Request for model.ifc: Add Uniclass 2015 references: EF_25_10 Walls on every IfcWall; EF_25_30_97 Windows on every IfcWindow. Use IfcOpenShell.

First a look at what the model holds.

```python
import ifcopenshell

model = ifcopenshell.open("model.ifc")
print(model.schema)
print("classifications:", [c.Name for c in model.by_type("IfcClassification")])
for ifc_class in ("IfcDoor", "IfcRoof", "IfcStair", "IfcWall", "IfcWindow"):
    print(ifc_class, len(model.by_type(ifc_class)))
```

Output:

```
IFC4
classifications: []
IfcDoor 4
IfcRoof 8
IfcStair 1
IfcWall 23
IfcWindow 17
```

```python
import ifcopenshell
import ifcopenshell.api.classification

model = ifcopenshell.open("model.ifc")

system = ifcopenshell.api.classification.add_classification(model, classification="Uniclass 2015")

codes = {
    "IfcWall": ("EF_25_10", "Walls"),
    "IfcWindow": ("EF_25_30_97", "Windows"),
}
for ifc_class, (code, name) in codes.items():
    products = model.by_type(ifc_class)
    ifcopenshell.api.classification.add_reference(
        model, products=products, classification=system, identification=code, name=name
    )
    print(code, len(products))

model.write("model_v2.ifc")
```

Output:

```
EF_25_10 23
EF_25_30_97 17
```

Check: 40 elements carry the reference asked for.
